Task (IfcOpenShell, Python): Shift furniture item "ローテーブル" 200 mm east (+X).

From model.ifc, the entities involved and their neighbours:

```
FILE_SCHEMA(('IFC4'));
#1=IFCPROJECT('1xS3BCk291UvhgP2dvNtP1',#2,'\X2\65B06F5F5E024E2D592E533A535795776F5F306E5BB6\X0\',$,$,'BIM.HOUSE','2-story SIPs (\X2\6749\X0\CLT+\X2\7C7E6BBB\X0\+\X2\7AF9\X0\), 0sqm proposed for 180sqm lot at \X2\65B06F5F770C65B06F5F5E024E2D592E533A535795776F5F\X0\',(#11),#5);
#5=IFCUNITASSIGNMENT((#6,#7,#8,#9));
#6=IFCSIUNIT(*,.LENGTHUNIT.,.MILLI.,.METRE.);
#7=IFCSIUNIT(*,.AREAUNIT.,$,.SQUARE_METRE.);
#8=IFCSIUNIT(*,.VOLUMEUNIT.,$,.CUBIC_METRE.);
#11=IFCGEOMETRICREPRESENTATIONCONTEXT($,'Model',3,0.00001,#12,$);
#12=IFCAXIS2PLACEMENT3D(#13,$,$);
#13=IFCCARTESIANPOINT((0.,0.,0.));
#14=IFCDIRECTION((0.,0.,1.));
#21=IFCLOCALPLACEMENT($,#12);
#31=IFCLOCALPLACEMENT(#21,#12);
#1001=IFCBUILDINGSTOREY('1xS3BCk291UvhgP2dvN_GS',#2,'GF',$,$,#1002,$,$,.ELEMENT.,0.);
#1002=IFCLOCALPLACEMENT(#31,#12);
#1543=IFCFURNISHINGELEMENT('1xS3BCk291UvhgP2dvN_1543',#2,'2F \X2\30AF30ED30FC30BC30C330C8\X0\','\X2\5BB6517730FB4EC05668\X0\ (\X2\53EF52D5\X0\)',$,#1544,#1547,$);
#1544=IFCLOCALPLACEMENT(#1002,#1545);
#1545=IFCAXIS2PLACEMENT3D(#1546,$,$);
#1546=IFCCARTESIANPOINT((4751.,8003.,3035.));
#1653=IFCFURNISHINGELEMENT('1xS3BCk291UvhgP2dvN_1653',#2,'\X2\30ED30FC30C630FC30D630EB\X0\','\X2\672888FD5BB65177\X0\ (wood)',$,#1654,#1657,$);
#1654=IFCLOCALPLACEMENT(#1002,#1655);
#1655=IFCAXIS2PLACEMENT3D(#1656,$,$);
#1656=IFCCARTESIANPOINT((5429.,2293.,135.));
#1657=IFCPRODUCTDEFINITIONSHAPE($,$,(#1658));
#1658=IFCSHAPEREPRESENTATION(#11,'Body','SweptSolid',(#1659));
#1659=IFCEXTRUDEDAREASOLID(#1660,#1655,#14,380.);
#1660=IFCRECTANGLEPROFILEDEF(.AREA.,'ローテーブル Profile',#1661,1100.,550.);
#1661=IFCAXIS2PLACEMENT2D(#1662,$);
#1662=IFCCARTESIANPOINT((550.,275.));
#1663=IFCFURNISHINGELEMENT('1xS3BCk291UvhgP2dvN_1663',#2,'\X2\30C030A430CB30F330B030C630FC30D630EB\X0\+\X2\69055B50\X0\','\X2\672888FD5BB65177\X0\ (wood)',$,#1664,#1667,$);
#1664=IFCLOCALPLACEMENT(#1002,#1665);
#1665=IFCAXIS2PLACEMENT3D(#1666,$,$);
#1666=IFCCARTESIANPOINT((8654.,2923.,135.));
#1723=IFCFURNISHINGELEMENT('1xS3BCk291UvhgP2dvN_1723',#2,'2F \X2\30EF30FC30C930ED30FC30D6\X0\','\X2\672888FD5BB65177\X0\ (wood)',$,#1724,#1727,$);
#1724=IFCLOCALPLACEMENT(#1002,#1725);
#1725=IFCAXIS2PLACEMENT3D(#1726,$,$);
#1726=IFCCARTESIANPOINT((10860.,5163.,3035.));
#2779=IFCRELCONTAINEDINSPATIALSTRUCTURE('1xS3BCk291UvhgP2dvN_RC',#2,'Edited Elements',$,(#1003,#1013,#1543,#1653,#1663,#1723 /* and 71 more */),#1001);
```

```python
import ifcopenshell
import ifcopenshell.api.geometry
import ifcopenshell.util.placement

model = ifcopenshell.open("model.ifc")

item = model.by_guid("1xS3BCk291UvhgP2dvN_1653")
matrix = ifcopenshell.util.placement.get_local_placement(item.ObjectPlacement)
matrix[0, 3] += 200.0
ifcopenshell.api.geometry.edit_object_placement(model, product=item, matrix=matrix, is_si=False)

print(ifcopenshell.util.placement.get_local_placement(item.ObjectPlacement).round(3) + 0.0)

model.write("model_v2.ifc")
```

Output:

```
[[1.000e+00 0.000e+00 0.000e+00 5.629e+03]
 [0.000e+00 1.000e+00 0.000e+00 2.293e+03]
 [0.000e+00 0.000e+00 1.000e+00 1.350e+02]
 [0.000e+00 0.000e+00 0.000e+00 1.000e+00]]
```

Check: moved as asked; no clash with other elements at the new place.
